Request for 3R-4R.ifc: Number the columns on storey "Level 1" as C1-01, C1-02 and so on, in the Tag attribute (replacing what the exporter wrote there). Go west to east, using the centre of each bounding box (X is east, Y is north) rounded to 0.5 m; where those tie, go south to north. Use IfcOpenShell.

First a look at what the model holds.

```python
import ifcopenshell
import ifcopenshell.util.element
import ifcopenshell.util.placement

model = ifcopenshell.open("3R-4R.ifc")
print(model.schema)
storey = next(s for s in model.by_type("IfcBuildingStorey") if s.Name == "Level 1")
columns = [e for e in ifcopenshell.util.element.get_decomposition(storey) if e.is_a("IfcColumn")]
for e in sorted(columns, key=lambda e: e.id()):
    origin = ifcopenshell.util.placement.get_local_placement(e.ObjectPlacement)[:3, 3]
    print(e.id(), e.Tag, e.Name, origin.round(2) + 0.0, sep=" | ")
```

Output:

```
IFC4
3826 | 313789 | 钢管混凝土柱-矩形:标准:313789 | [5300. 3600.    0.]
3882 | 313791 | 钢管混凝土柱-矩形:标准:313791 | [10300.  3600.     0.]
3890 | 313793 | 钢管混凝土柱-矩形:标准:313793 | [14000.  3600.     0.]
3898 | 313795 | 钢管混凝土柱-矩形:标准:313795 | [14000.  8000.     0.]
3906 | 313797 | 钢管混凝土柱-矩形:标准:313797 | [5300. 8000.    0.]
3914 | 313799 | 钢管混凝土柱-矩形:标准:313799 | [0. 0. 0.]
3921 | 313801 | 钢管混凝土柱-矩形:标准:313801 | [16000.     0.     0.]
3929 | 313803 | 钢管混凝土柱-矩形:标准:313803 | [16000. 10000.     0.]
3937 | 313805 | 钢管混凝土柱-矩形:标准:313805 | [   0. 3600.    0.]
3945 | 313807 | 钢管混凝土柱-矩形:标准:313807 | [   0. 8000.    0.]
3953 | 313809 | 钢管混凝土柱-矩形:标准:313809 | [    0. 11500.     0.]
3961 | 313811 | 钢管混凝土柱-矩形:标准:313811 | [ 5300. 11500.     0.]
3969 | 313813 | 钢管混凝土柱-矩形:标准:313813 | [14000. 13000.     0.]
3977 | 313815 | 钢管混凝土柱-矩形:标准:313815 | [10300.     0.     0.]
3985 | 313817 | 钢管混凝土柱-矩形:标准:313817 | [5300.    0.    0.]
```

```python
import ifcopenshell
import ifcopenshell.geom
import ifcopenshell.util.element
import ifcopenshell.util.shape

model = ifcopenshell.open("3R-4R.ifc")
settings = ifcopenshell.geom.settings()
settings.set("use-world-coords", True)


def centre(element):
    shape = ifcopenshell.geom.create_shape(settings, element)
    return ifcopenshell.util.shape.get_bbox_centroid(shape.geometry)


storey = next(s for s in model.by_type("IfcBuildingStorey") if s.Name == "Level 1")
columns = [e for e in ifcopenshell.util.element.get_decomposition(storey) if e.is_a("IfcColumn")]

# Insertion points can sit at a corner or the storey origin, so sort by the geometry (in metres).
centres = {e: centre(e) for e in columns}
columns.sort(key=lambda e: (round(centres[e][0] / 0.5), centres[e][1]))

for i, e in enumerate(columns, start=1):
    number = f"C1-{i:02d}"
    e.Tag = number
    print(e.id(), number)

model.write("3R-4R-out.ifc")
```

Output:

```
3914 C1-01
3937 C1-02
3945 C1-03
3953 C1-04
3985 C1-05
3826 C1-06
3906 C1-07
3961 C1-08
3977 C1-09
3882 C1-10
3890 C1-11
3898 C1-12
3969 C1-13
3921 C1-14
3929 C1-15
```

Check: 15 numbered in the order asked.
